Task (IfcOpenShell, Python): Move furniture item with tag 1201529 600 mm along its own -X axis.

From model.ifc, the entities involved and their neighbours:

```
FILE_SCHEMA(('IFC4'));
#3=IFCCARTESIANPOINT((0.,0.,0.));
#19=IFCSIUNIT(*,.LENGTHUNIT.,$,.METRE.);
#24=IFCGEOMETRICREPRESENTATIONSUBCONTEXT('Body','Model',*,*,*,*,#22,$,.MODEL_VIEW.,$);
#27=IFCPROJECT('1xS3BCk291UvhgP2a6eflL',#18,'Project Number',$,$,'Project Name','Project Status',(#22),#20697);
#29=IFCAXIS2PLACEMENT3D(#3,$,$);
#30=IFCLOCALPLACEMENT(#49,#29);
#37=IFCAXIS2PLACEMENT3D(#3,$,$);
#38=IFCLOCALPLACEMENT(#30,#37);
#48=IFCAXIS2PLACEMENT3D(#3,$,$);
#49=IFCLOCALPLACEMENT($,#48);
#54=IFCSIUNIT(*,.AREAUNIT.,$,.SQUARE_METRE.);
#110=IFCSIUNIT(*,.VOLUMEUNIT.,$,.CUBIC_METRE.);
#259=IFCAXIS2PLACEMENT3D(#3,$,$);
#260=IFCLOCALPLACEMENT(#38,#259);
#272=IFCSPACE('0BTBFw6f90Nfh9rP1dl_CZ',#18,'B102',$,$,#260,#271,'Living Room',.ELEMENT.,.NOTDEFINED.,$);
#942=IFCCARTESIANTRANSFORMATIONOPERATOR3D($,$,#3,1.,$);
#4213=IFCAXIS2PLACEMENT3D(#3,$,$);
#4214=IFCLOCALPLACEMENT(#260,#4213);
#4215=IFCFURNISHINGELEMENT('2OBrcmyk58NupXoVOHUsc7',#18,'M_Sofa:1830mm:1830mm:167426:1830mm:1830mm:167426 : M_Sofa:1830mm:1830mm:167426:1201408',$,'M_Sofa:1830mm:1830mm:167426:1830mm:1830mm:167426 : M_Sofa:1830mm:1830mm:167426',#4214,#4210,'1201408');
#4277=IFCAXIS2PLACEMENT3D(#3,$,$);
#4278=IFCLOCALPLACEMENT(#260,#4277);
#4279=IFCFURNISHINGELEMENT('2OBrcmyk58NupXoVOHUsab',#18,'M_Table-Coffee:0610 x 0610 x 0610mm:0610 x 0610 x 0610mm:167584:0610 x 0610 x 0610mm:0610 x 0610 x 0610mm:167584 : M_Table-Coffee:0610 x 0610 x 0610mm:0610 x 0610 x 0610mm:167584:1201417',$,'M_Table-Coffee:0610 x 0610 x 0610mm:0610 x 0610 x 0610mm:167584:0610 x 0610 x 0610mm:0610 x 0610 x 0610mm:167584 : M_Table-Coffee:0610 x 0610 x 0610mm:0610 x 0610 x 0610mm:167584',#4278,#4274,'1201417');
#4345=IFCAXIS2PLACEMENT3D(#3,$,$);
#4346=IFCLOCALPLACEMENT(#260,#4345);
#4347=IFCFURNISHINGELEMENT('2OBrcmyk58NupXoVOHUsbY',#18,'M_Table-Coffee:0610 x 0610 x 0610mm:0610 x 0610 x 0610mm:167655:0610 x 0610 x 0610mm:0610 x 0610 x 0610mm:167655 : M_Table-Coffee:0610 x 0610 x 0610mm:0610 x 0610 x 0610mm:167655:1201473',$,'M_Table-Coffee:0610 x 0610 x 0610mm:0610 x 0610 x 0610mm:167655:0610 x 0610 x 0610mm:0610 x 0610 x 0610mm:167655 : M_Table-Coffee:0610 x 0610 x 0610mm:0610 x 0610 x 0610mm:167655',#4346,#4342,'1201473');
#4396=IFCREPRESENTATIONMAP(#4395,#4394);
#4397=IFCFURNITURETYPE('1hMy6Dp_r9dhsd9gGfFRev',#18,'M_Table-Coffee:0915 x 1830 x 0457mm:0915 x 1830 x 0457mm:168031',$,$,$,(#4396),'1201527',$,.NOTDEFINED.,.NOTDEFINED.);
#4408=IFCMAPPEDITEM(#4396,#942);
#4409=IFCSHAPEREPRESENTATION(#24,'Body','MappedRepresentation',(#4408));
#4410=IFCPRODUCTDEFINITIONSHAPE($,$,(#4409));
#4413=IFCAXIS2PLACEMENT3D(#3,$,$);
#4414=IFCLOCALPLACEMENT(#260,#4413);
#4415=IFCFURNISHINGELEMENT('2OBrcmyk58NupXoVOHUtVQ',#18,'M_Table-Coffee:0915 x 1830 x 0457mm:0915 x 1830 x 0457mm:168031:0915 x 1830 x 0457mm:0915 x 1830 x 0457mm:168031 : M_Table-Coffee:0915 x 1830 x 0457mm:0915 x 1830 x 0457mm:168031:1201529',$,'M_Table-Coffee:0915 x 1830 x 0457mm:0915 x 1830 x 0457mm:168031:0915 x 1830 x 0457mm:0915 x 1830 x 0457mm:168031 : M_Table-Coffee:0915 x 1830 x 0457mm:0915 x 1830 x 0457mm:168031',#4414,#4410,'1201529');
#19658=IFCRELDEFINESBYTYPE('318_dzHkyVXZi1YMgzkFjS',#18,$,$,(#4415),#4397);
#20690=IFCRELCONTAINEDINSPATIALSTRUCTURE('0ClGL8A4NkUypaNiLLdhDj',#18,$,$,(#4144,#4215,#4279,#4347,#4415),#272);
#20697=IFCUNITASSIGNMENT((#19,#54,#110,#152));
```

```python
import ifcopenshell
import ifcopenshell.api.geometry
import ifcopenshell.util.placement
import ifcopenshell.util.unit

model = ifcopenshell.open("model.ifc")
unit_scale = ifcopenshell.util.unit.calculate_unit_scale(model)

item = model.by_id(4415)
matrix = ifcopenshell.util.placement.get_local_placement(item.ObjectPlacement)
matrix[:3, 3] -= matrix[:3, 0] * 0.6 / unit_scale
ifcopenshell.api.geometry.edit_object_placement(model, product=item, matrix=matrix, is_si=False)

print(ifcopenshell.util.placement.get_local_placement(item.ObjectPlacement).round(3) + 0.0)

model.write("model_rev.ifc")
```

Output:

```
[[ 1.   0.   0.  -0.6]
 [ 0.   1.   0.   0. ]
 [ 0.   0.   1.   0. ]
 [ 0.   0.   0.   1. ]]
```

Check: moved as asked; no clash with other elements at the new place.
